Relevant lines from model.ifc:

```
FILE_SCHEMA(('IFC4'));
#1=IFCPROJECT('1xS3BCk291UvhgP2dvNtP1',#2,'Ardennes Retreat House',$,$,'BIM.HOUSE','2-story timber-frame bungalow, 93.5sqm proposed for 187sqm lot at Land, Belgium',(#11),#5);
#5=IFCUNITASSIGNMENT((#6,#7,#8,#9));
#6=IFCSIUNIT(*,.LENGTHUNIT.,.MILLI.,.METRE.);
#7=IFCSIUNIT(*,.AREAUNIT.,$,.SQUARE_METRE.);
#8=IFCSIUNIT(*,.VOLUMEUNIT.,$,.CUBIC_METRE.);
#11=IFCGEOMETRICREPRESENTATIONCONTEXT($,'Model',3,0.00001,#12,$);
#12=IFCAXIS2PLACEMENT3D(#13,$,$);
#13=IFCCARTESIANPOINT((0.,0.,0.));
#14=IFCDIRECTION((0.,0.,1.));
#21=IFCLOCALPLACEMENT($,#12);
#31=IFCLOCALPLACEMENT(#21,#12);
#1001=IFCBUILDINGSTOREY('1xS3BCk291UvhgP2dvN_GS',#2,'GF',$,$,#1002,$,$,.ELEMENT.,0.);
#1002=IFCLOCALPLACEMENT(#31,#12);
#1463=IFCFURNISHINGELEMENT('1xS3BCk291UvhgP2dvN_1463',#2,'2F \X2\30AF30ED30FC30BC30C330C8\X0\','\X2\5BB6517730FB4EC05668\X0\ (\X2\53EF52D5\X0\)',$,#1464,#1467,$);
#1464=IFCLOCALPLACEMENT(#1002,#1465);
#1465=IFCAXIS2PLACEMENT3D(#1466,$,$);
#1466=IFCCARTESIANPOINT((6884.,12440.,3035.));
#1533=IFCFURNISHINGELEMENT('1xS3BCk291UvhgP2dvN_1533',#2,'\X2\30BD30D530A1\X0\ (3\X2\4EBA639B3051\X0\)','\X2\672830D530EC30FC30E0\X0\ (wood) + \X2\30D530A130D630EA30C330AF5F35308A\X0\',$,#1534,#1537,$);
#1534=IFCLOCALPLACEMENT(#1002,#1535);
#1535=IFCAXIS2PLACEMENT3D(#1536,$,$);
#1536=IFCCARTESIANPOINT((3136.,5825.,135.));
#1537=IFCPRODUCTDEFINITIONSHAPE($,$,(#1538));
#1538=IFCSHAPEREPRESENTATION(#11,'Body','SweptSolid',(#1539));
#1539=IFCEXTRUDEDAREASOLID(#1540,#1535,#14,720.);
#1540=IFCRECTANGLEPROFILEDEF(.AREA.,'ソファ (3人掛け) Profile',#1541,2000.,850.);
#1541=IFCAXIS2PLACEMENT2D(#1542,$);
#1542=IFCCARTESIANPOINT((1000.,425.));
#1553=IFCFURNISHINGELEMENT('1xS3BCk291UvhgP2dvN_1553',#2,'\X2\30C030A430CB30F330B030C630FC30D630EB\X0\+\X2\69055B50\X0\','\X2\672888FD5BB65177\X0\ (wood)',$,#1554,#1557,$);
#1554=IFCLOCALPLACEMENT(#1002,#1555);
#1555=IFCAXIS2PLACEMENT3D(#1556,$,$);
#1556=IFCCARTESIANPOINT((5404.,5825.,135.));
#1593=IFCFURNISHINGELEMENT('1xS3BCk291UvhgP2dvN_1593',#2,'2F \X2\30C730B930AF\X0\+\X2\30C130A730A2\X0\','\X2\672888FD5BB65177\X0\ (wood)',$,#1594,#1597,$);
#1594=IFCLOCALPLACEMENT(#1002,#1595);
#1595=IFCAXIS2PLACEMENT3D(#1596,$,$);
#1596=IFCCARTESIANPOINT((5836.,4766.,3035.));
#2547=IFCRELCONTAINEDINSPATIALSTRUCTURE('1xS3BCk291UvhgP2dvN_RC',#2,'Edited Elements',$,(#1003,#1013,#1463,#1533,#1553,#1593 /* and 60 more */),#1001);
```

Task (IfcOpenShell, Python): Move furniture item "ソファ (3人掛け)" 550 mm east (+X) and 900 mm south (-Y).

```python
import ifcopenshell
import ifcopenshell.api.geometry
import ifcopenshell.util.placement
import ifcopenshell.util.unit

model = ifcopenshell.open("model.ifc")
unit_scale = ifcopenshell.util.unit.calculate_unit_scale(model)

item = model.by_guid("1xS3BCk291UvhgP2dvN_1533")
matrix = ifcopenshell.util.placement.get_local_placement(item.ObjectPlacement)
matrix[0, 3] += 0.55 / unit_scale
matrix[1, 3] -= 0.9 / unit_scale
ifcopenshell.api.geometry.edit_object_placement(model, product=item, matrix=matrix, is_si=False)

print(ifcopenshell.util.placement.get_local_placement(item.ObjectPlacement).round(3) + 0.0)

model.write("model-out.ifc")
```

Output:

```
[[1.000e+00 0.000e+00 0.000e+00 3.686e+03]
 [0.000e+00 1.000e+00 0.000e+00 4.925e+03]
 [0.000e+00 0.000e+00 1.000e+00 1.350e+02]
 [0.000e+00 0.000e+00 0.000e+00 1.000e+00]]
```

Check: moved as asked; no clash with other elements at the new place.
